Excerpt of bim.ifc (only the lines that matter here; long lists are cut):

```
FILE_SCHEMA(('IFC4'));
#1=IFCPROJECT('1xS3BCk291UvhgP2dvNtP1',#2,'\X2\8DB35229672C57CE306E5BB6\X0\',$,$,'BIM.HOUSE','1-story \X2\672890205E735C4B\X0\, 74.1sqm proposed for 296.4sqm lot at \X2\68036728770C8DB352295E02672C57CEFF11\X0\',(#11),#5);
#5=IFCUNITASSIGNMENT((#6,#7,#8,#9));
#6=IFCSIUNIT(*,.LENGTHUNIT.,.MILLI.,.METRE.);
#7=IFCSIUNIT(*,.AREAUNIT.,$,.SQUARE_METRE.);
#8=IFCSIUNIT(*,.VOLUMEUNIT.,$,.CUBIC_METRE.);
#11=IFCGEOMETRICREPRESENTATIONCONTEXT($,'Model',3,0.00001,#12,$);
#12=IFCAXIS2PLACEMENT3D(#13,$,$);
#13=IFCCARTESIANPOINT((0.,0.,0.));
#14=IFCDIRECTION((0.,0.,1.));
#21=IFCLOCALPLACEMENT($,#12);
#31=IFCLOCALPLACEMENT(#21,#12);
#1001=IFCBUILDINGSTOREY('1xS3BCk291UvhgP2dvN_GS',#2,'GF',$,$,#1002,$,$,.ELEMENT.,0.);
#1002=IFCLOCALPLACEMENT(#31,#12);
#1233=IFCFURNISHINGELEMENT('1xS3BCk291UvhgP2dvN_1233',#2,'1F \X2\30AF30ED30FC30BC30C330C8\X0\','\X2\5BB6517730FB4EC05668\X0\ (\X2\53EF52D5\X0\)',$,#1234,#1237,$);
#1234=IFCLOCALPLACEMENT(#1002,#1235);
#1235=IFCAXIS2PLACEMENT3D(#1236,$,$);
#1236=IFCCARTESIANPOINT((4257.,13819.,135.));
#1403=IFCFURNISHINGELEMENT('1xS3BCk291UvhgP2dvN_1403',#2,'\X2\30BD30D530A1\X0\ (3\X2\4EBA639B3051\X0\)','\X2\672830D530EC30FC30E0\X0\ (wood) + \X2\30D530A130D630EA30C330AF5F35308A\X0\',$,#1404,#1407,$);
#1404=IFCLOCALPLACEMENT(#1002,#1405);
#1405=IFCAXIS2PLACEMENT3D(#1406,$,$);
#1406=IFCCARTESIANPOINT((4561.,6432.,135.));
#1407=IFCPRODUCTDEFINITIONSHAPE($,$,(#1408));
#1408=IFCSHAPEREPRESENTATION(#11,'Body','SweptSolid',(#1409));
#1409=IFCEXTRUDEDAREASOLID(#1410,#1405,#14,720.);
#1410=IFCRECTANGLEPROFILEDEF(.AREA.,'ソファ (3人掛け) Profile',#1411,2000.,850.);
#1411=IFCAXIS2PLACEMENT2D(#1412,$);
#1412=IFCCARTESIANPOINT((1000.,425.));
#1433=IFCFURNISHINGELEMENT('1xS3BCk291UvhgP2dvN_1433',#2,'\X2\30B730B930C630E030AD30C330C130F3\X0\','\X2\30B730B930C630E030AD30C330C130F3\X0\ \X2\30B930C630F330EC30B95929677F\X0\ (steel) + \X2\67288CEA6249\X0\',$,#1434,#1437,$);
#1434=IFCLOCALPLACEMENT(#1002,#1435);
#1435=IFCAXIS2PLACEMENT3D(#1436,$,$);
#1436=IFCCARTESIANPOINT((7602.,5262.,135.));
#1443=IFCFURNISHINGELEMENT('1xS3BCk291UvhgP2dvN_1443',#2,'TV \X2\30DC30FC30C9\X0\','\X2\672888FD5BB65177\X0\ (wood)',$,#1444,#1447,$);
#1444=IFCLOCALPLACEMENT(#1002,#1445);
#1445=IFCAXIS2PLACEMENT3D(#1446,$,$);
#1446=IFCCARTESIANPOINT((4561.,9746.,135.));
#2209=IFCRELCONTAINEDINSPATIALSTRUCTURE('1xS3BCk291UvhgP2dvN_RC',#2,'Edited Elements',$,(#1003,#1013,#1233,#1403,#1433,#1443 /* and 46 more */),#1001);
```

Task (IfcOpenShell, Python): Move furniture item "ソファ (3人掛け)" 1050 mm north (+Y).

```python
import ifcopenshell
import ifcopenshell.api.geometry
import ifcopenshell.util.placement
import ifcopenshell.util.unit

model = ifcopenshell.open("bim.ifc")
unit_scale = ifcopenshell.util.unit.calculate_unit_scale(model)

item = model.by_id(1403)
matrix = ifcopenshell.util.placement.get_local_placement(item.ObjectPlacement)
matrix[1, 3] += 1.05 / unit_scale
ifcopenshell.api.geometry.edit_object_placement(model, product=item, matrix=matrix, is_si=False)

print(ifcopenshell.util.placement.get_local_placement(item.ObjectPlacement).round(3) + 0.0)

model.write("bim_rev.ifc")
```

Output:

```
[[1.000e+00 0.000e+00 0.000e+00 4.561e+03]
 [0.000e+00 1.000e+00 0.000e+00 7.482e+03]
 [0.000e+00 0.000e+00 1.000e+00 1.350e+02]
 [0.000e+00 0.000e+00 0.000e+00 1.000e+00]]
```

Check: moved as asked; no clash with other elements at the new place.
